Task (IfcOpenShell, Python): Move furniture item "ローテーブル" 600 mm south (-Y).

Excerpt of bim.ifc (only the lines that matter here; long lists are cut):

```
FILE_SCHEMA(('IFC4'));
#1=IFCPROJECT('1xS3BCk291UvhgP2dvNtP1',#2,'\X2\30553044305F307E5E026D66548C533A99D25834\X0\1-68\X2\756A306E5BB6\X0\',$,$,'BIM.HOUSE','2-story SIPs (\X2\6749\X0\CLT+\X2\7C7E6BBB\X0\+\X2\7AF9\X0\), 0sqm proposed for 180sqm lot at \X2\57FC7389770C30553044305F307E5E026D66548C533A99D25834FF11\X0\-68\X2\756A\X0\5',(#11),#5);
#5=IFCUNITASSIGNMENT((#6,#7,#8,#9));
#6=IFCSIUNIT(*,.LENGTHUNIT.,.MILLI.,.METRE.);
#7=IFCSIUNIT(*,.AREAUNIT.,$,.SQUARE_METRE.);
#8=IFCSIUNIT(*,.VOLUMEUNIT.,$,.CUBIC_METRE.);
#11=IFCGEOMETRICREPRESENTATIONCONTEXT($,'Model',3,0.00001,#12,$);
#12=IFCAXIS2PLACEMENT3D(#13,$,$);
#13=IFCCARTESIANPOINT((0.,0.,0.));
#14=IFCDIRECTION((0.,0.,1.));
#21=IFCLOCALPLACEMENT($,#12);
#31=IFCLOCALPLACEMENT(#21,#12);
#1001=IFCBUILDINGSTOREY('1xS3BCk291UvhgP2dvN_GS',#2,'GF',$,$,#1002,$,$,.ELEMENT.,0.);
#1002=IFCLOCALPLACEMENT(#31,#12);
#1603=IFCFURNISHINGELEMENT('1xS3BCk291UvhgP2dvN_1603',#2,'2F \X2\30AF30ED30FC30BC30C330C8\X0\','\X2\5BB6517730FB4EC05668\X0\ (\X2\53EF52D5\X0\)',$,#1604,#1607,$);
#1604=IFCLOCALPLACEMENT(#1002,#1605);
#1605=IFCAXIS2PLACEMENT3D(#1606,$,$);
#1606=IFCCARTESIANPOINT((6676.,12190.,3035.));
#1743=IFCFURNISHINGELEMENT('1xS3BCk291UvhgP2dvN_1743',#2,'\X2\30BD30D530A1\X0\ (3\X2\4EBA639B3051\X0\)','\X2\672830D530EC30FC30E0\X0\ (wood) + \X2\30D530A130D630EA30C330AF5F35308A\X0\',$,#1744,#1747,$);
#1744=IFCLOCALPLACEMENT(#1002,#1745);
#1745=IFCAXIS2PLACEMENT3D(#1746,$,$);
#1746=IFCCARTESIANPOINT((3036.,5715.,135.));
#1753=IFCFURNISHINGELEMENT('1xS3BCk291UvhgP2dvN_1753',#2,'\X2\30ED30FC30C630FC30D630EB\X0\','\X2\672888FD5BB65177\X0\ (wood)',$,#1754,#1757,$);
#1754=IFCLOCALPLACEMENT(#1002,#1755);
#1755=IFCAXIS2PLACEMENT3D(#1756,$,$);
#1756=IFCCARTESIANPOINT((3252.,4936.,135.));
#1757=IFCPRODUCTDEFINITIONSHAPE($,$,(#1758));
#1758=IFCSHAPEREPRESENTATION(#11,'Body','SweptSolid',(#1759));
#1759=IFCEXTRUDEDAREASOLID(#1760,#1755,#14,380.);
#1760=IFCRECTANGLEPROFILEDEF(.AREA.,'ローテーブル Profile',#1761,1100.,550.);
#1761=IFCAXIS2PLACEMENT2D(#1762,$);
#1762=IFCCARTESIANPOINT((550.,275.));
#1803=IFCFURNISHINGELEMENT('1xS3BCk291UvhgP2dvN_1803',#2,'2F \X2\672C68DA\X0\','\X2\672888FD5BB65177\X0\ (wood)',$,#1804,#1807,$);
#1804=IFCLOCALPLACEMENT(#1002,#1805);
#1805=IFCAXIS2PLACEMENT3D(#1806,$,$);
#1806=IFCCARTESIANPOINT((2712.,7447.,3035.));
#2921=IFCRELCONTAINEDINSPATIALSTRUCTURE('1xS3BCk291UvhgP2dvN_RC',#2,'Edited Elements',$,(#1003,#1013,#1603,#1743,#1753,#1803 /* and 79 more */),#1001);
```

```python
import ifcopenshell
import ifcopenshell.api.geometry
import ifcopenshell.util.placement

model = ifcopenshell.open("bim.ifc")

item = model.by_id(1753)
matrix = ifcopenshell.util.placement.get_local_placement(item.ObjectPlacement)
matrix[1, 3] -= 600.0
ifcopenshell.api.geometry.edit_object_placement(model, product=item, matrix=matrix, is_si=False)

print(ifcopenshell.util.placement.get_local_placement(item.ObjectPlacement).round(3) + 0.0)

model.write("bim_updated.ifc")
```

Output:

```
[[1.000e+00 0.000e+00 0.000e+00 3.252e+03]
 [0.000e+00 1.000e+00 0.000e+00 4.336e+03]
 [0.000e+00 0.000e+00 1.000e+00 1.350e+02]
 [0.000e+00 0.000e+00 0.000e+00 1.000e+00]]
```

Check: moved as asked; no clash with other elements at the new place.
